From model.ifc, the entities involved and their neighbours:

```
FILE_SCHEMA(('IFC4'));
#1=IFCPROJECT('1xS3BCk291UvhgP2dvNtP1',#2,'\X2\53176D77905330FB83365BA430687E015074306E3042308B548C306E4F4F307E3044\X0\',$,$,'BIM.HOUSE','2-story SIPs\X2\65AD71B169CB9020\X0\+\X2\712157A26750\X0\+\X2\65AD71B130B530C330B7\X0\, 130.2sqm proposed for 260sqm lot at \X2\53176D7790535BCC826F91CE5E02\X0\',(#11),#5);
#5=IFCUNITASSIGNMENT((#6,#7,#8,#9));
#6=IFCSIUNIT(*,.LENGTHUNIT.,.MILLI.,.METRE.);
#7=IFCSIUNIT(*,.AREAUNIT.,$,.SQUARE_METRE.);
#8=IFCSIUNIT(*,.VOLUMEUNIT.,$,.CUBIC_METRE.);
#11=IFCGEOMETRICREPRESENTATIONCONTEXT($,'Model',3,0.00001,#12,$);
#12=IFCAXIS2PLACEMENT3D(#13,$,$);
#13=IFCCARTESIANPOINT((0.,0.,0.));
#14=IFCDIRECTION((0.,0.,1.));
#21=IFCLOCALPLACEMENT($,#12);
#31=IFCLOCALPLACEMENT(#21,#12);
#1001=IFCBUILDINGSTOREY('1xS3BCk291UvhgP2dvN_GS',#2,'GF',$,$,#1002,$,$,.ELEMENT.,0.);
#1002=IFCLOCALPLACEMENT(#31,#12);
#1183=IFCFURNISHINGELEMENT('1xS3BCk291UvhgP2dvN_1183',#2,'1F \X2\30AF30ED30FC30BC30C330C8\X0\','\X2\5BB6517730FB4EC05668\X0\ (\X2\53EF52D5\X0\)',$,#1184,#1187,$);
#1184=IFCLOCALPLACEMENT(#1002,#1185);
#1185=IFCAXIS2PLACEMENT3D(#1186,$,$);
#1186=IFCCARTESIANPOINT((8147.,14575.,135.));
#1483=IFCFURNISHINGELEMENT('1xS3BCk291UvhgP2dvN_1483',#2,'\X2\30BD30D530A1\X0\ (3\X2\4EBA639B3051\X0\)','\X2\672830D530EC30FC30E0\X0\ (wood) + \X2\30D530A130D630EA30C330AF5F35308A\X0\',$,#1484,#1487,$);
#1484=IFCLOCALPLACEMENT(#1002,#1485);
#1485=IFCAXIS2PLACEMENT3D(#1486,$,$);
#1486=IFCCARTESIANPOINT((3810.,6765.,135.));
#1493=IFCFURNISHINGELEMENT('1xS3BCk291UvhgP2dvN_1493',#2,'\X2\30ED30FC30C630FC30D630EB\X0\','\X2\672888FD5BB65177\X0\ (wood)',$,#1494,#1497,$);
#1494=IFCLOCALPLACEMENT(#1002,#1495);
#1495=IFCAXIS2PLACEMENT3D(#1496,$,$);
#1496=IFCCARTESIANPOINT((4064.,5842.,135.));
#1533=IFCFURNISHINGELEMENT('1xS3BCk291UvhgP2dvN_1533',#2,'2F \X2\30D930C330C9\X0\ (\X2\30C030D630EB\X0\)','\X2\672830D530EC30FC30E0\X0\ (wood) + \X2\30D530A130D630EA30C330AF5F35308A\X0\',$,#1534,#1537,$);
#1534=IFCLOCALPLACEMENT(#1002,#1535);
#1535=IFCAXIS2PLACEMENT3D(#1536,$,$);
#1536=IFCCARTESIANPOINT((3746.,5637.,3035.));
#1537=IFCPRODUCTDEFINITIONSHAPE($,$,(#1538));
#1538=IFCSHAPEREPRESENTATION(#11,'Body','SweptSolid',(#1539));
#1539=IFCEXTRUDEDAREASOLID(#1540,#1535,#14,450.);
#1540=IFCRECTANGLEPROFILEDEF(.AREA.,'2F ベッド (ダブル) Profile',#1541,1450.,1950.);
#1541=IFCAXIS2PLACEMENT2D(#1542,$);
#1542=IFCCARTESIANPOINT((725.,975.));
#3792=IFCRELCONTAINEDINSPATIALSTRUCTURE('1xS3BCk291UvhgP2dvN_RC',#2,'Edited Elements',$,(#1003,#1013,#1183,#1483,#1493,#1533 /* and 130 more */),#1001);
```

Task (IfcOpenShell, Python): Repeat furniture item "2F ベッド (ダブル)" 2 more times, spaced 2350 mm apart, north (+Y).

```python
import numpy as np
import ifcopenshell
import ifcopenshell.api.geometry
import ifcopenshell.api.root
import ifcopenshell.util.element
import ifcopenshell.util.placement

model = ifcopenshell.open("model.ifc")


def reuse_history(source, copy):
    """copy_class also copies each property set's owner history, people and application; keep the originals."""
    for rel in copy.IsDefinedBy:
        if rel.is_a("IfcRelDefinesByProperties") and (history := rel.RelatingPropertyDefinition.OwnerHistory):
            rel.RelatingPropertyDefinition.OwnerHistory = source.OwnerHistory
            ifcopenshell.util.element.remove_deep2(model, history)


source = model.by_guid("1xS3BCk291UvhgP2dvN_1533")
base = ifcopenshell.util.placement.get_local_placement(source.ObjectPlacement)
step = np.array([0.0, 1.0, 0.0]) * 2350.0

for i in range(1, 3):
    copy = ifcopenshell.api.root.copy_class(model, product=source)
    copy.Representation = ifcopenshell.util.element.copy_deep(
        model, source.Representation, exclude=["IfcGeometricRepresentationContext", "IfcRepresentationMap"]
    )
    reuse_history(source, copy)
    matrix = base.copy()
    matrix[:3, 3] += i * step
    print("added at", matrix[:3, 3].round(3) + 0.0)
    ifcopenshell.api.geometry.edit_object_placement(model, product=copy, matrix=matrix, is_si=False)

model.write("model_v2.ifc")
```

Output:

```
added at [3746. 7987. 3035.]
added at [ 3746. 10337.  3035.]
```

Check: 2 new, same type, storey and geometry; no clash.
